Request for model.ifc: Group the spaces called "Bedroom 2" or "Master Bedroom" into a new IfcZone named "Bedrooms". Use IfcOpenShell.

First a look at what the model holds.

```python
import ifcopenshell

model = ifcopenshell.open("model.ifc")
print(model.schema)
seen = {}
for space in model.by_type("IfcSpace"):
    seen[space.LongName] = seen.get(space.LongName, 0) + 1
for name, count in sorted(seen.items(), key=str):
    print(count, "x", name)
print("zones:", [z.Name for z in model.by_type("IfcZone")][:20])
```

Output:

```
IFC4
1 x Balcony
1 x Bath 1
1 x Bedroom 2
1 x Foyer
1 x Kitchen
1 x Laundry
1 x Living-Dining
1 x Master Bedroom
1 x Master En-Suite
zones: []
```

```python
import ifcopenshell
import ifcopenshell.api.group
import ifcopenshell.api.root

model = ifcopenshell.open("model.ifc")

names = {"Bedroom 2", "Master Bedroom"}
spaces = [s for s in model.by_type("IfcSpace") if s.LongName in names]

zone = ifcopenshell.api.root.create_entity(model, ifc_class="IfcZone", name="Bedrooms")
ifcopenshell.api.group.assign_group(model, products=spaces, group=zone)
print(len(spaces), "spaces in", zone.Name)

model.write("model_v2.ifc")
```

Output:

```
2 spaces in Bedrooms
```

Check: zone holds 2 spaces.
